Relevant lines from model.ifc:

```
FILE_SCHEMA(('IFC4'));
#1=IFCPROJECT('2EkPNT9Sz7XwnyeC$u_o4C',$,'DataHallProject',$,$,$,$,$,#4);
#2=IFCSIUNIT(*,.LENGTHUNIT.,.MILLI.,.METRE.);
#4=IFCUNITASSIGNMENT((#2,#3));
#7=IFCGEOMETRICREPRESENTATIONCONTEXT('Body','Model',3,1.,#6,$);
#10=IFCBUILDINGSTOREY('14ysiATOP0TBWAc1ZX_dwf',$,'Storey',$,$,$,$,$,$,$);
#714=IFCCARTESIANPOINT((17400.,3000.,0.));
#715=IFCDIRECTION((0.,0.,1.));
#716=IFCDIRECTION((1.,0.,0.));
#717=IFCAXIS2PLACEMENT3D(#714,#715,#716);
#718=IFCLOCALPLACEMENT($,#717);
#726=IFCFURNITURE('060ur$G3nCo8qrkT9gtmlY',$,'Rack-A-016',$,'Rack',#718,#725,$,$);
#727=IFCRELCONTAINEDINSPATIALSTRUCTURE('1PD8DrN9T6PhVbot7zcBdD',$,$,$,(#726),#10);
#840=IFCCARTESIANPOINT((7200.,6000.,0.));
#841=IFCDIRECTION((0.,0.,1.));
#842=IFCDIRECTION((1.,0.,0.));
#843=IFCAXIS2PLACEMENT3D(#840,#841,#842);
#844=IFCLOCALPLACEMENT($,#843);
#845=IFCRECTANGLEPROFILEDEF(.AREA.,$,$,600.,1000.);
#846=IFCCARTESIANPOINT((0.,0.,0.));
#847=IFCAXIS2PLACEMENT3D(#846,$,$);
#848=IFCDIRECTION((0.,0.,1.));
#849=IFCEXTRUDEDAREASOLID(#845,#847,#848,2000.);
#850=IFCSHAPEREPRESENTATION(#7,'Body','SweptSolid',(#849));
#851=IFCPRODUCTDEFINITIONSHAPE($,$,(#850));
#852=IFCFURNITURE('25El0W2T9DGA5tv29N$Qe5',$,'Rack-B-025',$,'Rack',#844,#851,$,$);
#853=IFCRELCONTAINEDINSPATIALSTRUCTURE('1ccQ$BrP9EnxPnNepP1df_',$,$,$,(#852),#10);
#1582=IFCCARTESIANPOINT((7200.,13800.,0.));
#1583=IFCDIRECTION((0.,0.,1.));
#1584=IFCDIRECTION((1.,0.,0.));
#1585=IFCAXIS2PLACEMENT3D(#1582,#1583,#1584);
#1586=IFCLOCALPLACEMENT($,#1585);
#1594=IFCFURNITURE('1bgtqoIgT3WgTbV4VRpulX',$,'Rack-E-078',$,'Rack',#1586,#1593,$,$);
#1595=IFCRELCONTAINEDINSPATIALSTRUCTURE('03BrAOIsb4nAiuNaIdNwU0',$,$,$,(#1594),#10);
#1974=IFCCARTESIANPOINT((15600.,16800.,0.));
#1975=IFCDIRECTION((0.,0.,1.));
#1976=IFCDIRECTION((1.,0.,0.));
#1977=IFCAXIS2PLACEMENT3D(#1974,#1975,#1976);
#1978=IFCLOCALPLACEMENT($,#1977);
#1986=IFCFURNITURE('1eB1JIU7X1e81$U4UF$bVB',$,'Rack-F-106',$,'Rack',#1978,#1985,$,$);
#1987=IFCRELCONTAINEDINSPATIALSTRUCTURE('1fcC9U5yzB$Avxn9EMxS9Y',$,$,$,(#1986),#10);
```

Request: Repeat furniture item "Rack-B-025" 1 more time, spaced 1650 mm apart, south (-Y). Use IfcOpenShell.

```python
import numpy as np
import ifcopenshell
import ifcopenshell.api.geometry
import ifcopenshell.api.root
import ifcopenshell.util.element
import ifcopenshell.util.placement
import ifcopenshell.util.unit

model = ifcopenshell.open("model.ifc")
unit_scale = ifcopenshell.util.unit.calculate_unit_scale(model)

source = model.by_guid("25El0W2T9DGA5tv29N$Qe5")
base = ifcopenshell.util.placement.get_local_placement(source.ObjectPlacement)
step = np.array([0.0, -1.0, 0.0]) * 1.65 / unit_scale

for i in range(1, 2):
    copy = ifcopenshell.api.root.copy_class(model, product=source)
    copy.Representation = ifcopenshell.util.element.copy_deep(
        model, source.Representation, exclude=["IfcGeometricRepresentationContext", "IfcRepresentationMap"]
    )
    matrix = base.copy()
    matrix[:3, 3] += i * step
    print("added at", matrix[:3, 3].round(3) + 0.0)
    ifcopenshell.api.geometry.edit_object_placement(model, product=copy, matrix=matrix, is_si=False)

model.write("model_rev.ifc")
```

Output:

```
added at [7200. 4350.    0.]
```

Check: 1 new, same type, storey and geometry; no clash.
